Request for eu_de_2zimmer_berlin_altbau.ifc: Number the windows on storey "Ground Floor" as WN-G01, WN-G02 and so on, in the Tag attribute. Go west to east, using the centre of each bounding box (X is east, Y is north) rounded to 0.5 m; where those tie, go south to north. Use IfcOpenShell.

First a look at what the model holds.

```python
import ifcopenshell
import ifcopenshell.util.element
import ifcopenshell.util.placement

model = ifcopenshell.open("eu_de_2zimmer_berlin_altbau.ifc")
print(model.schema)
storey = next(s for s in model.by_type("IfcBuildingStorey") if s.Name == "Ground Floor")
windows = [e for e in ifcopenshell.util.element.get_decomposition(storey) if e.is_a("IfcWindow")]
for e in sorted(windows, key=lambda e: e.id()):
    origin = ifcopenshell.util.placement.get_local_placement(e.ObjectPlacement)[:3, 3]
    print(e.id(), e.Tag, e.Name, origin.round(2) + 0.0, sep=" | ")
```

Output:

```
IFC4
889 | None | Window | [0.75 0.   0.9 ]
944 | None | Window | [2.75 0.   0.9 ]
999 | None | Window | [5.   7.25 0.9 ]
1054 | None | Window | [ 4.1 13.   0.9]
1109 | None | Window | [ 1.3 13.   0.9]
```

```python
import ifcopenshell
import ifcopenshell.geom
import ifcopenshell.util.element
import ifcopenshell.util.shape

model = ifcopenshell.open("eu_de_2zimmer_berlin_altbau.ifc")
settings = ifcopenshell.geom.settings()
settings.set("use-world-coords", True)


def centre(element):
    shape = ifcopenshell.geom.create_shape(settings, element)
    return ifcopenshell.util.shape.get_bbox_centroid(shape.geometry)


storey = next(s for s in model.by_type("IfcBuildingStorey") if s.Name == "Ground Floor")
windows = [e for e in ifcopenshell.util.element.get_decomposition(storey) if e.is_a("IfcWindow")]

# Insertion points can sit at a corner or the storey origin, so sort by the geometry (in metres).
centres = {e: centre(e) for e in windows}
windows.sort(key=lambda e: (round(centres[e][0] / 0.5), centres[e][1]))

for i, e in enumerate(windows, start=1):
    number = f"WN-G{i:02d}"
    e.Tag = number
    print(e.id(), number)

model.write("eu_de_2zimmer_berlin_altbau_v2.ifc")
```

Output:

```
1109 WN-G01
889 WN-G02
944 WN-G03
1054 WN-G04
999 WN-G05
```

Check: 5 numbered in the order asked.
